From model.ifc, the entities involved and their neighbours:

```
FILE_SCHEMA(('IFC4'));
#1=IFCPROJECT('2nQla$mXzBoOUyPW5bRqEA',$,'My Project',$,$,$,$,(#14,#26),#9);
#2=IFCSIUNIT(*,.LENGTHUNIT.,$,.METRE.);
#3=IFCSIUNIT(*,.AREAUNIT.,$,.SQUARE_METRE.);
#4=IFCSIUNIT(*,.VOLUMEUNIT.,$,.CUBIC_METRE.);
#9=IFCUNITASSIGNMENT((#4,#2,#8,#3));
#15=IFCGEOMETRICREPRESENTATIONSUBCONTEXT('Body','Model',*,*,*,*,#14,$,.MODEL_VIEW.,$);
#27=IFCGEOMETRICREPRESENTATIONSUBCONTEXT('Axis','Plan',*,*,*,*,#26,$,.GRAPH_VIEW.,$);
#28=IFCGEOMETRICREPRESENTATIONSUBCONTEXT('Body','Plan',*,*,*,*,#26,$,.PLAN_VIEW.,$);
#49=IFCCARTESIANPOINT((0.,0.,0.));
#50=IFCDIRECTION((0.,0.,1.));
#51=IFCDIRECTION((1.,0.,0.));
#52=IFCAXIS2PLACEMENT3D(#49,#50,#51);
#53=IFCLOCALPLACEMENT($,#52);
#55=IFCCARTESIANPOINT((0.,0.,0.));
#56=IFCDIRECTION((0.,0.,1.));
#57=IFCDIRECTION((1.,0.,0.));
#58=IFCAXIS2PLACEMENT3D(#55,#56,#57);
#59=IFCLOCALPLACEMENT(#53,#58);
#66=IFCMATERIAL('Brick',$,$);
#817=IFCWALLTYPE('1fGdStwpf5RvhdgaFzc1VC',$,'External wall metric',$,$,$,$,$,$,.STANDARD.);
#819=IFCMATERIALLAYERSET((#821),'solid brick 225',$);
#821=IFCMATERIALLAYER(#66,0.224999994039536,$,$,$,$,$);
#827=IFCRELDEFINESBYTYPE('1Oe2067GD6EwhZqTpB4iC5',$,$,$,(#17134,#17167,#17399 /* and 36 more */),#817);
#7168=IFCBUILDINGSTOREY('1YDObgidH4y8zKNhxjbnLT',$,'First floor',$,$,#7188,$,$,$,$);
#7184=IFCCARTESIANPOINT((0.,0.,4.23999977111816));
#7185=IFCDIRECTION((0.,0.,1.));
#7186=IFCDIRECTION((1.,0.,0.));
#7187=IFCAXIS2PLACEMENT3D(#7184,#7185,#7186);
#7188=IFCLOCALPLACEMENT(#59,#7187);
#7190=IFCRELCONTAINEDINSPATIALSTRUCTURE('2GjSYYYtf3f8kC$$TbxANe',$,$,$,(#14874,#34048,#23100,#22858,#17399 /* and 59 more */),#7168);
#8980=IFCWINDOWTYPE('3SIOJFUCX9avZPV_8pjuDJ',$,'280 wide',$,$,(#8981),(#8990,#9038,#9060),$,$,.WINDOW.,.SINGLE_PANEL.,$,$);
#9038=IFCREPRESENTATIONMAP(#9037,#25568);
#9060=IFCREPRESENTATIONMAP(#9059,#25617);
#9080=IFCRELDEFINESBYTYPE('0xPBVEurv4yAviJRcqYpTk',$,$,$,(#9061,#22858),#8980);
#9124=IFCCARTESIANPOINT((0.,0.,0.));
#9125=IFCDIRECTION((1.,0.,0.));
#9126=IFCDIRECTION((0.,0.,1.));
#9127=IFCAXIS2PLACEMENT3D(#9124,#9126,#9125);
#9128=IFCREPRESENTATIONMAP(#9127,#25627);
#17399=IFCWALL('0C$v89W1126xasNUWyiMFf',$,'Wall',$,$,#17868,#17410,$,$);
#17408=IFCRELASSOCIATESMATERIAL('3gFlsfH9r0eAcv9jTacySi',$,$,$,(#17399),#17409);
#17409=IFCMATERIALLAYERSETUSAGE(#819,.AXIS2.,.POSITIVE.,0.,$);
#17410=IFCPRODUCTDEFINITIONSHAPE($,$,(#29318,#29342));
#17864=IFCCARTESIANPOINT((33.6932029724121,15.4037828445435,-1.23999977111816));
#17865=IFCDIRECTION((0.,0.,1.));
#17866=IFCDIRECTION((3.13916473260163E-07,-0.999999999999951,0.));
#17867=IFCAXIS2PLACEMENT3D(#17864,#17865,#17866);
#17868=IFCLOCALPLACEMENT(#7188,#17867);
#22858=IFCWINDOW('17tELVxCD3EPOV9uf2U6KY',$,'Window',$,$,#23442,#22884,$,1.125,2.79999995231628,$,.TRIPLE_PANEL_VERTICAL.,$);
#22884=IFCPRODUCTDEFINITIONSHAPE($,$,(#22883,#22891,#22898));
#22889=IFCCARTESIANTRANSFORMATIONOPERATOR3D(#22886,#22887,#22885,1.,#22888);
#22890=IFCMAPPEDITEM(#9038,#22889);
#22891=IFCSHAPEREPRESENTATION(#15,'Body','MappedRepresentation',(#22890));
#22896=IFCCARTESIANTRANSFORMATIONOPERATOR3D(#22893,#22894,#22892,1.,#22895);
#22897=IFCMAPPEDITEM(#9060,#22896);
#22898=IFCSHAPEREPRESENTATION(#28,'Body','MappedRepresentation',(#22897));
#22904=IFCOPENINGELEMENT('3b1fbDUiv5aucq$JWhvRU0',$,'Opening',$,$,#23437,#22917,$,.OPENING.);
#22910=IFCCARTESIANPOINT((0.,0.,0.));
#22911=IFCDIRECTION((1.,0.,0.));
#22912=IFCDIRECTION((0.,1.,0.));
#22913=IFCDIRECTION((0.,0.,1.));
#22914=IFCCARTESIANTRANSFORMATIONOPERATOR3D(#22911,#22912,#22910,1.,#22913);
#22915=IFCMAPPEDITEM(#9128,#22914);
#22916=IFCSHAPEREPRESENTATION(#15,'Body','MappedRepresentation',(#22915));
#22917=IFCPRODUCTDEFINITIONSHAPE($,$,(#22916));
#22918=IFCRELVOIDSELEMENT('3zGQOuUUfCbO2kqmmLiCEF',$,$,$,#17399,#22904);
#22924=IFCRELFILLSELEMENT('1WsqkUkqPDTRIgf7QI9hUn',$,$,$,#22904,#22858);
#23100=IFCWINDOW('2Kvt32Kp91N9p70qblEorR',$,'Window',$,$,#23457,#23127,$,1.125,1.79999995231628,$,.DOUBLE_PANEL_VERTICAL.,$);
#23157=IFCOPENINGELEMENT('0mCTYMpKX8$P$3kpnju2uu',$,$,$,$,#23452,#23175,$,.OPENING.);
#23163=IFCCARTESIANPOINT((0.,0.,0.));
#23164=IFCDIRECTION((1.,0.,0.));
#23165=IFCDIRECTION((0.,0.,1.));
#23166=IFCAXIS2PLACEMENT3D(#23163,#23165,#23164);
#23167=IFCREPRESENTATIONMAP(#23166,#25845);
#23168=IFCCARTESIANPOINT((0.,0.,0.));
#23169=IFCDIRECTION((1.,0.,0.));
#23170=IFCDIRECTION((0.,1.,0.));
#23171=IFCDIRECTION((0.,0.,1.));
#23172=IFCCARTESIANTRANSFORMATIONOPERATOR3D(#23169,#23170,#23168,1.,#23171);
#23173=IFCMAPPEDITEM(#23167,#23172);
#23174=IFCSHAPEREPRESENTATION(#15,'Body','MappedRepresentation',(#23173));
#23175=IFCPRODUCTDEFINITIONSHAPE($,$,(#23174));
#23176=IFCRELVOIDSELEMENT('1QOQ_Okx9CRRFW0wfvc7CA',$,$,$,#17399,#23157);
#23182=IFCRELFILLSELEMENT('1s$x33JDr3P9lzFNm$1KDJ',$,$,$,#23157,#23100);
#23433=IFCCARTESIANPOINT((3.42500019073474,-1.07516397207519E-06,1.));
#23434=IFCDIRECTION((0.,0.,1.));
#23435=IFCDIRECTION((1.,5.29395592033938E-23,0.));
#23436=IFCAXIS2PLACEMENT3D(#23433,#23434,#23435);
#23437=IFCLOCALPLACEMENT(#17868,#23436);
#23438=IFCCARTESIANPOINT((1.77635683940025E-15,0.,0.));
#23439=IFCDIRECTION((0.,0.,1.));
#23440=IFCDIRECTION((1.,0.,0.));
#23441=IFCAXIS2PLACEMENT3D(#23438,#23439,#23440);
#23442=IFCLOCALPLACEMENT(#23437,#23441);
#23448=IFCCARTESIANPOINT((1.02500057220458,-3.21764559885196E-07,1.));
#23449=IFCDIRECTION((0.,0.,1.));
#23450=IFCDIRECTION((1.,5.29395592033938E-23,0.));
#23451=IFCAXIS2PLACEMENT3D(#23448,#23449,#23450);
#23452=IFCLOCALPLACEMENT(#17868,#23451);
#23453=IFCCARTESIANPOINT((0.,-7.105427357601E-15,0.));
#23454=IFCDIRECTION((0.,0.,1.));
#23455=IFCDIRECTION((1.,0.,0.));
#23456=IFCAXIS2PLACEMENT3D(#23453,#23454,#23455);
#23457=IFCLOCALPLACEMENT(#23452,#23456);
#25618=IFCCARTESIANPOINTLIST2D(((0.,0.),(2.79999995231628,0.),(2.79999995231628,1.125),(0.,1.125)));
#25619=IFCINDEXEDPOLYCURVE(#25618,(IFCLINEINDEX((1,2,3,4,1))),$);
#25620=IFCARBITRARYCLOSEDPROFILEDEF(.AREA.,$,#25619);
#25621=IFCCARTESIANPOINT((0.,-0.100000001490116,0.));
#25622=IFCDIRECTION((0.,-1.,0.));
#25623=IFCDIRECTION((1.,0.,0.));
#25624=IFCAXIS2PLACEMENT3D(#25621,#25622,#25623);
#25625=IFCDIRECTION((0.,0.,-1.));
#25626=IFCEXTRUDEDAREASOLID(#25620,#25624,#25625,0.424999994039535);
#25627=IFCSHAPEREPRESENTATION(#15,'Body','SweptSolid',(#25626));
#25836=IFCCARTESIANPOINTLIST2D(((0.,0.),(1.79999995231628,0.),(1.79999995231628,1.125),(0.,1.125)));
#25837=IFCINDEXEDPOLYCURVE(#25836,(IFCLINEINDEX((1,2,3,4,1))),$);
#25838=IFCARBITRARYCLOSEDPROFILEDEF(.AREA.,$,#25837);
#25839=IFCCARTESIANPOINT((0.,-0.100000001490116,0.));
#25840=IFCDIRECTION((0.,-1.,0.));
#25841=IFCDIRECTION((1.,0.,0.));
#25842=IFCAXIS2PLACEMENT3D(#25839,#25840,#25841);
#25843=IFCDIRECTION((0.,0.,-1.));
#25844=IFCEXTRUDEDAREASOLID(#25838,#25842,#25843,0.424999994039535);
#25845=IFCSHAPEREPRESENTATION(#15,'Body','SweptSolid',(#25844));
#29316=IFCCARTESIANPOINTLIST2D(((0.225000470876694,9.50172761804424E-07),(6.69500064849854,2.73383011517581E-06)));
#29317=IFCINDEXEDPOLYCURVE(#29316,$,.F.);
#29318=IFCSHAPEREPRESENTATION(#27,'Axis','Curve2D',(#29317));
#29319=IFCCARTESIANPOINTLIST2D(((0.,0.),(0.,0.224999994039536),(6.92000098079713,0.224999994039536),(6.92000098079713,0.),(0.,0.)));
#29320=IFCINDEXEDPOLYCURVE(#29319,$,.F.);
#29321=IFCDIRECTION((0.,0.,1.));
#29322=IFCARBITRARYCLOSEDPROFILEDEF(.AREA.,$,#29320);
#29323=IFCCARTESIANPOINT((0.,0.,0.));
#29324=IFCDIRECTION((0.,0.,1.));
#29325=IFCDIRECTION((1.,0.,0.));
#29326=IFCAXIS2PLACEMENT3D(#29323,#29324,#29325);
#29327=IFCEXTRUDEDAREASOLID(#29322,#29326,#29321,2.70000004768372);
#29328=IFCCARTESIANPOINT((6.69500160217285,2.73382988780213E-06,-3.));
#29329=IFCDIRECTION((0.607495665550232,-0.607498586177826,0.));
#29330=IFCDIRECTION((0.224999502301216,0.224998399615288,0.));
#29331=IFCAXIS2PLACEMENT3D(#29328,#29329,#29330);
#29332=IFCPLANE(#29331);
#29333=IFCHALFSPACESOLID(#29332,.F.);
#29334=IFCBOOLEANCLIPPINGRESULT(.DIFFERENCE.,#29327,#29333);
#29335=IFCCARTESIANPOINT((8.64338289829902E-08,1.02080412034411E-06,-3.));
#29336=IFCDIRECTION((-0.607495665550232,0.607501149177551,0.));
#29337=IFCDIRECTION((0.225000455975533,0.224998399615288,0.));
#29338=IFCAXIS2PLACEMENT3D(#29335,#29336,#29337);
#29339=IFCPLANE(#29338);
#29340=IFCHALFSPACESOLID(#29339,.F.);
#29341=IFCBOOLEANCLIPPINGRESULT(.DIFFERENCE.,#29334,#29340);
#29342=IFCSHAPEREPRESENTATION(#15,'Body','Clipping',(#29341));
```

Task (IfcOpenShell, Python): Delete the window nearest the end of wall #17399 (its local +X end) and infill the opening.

```python
import ifcopenshell
import ifcopenshell.api.feature
import ifcopenshell.api.root
import ifcopenshell.geom
import ifcopenshell.util.shape

model = ifcopenshell.open("model.ifc")
settings = ifcopenshell.geom.settings()


def volume(element):
    """Net volume in cubic metres, openings subtracted."""
    shape = ifcopenshell.geom.create_shape(settings, element)
    return ifcopenshell.util.shape.get_volume(shape.geometry)


window = model.by_guid("17tELVxCD3EPOV9uf2U6KY")
opening = window.FillsVoids[0].RelatingOpeningElement
wall = opening.VoidsElements[0].RelatingBuildingElement
before = volume(wall)

ifcopenshell.api.root.remove_product(model, product=window)
ifcopenshell.api.feature.remove_feature(model, feature=opening)

after = volume(wall)

print(f"wall volume {before:.3f} -> {after:.3f} m3")

model.write("model_edited.ifc")
```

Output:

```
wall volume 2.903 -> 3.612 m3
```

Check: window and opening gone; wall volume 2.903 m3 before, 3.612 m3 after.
